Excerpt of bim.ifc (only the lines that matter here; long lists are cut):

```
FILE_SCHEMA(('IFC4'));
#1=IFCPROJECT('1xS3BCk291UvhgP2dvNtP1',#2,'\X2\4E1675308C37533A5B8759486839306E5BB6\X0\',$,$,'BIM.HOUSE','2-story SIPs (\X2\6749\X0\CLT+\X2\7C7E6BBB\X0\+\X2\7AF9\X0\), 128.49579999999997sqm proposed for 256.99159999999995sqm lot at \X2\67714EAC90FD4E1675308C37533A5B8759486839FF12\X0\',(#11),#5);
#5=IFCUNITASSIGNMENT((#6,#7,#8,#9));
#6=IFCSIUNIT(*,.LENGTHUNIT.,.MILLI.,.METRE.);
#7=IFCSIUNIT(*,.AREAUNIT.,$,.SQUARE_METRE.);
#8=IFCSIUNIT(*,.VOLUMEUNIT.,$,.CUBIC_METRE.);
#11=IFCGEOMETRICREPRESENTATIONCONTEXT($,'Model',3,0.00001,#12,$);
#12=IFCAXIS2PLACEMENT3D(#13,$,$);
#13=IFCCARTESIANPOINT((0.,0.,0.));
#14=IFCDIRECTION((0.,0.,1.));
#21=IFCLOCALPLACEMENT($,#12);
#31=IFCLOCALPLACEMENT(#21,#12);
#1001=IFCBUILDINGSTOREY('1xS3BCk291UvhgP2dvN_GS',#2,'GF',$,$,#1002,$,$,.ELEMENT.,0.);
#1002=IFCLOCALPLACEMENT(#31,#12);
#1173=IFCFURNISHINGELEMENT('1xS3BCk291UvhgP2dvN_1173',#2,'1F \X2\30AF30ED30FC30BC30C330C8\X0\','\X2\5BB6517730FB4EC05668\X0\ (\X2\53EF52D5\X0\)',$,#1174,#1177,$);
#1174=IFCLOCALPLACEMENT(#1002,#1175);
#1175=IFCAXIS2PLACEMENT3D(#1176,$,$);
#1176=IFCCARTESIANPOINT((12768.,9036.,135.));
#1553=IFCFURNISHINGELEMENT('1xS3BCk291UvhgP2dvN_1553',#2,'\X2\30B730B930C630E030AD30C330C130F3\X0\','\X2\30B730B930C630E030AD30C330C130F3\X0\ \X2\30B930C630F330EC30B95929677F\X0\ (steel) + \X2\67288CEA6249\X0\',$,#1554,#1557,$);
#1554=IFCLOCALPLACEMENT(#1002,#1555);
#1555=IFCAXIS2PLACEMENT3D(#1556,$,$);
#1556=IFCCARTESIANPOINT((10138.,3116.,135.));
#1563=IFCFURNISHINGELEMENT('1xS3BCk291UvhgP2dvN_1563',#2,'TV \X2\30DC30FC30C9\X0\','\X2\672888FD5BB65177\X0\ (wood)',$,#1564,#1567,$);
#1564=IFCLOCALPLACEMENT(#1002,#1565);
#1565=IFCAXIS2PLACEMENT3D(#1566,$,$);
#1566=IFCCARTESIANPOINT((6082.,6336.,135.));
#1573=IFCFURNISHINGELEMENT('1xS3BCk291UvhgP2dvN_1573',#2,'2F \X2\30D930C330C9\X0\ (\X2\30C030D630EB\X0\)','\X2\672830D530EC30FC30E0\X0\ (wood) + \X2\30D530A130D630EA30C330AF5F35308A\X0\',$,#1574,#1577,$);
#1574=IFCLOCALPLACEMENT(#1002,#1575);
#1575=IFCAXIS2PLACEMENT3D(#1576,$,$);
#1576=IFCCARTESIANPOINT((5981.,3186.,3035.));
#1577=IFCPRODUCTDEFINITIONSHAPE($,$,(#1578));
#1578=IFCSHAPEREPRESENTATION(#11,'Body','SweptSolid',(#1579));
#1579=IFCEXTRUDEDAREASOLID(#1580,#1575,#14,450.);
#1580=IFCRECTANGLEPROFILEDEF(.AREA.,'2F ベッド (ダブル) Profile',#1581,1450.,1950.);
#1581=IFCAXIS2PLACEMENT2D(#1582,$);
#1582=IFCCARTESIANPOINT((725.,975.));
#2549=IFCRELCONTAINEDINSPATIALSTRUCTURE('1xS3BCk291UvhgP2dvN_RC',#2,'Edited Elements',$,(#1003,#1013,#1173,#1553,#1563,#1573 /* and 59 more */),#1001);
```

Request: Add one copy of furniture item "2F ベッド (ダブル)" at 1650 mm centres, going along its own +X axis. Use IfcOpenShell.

```python
import ifcopenshell
import ifcopenshell.api.geometry
import ifcopenshell.api.root
import ifcopenshell.util.element
import ifcopenshell.util.placement

model = ifcopenshell.open("bim.ifc")


def reuse_history(source, copy):
    """copy_class also copies each property set's owner history, people and application; keep the originals."""
    for rel in copy.IsDefinedBy:
        if rel.is_a("IfcRelDefinesByProperties") and (history := rel.RelatingPropertyDefinition.OwnerHistory):
            rel.RelatingPropertyDefinition.OwnerHistory = source.OwnerHistory
            ifcopenshell.util.element.remove_deep2(model, history)


source = model.by_id(1573)
base = ifcopenshell.util.placement.get_local_placement(source.ObjectPlacement)
step = base[:3, 0] * 1650.0

for i in range(1, 2):
    copy = ifcopenshell.api.root.copy_class(model, product=source)
    copy.Representation = ifcopenshell.util.element.copy_deep(
        model, source.Representation, exclude=["IfcGeometricRepresentationContext", "IfcRepresentationMap"]
    )
    reuse_history(source, copy)
    matrix = base.copy()
    matrix[:3, 3] += i * step
    print("added at", matrix[:3, 3].round(3) + 0.0)
    ifcopenshell.api.geometry.edit_object_placement(model, product=copy, matrix=matrix, is_si=False)

model.write("bim_updated.ifc")
```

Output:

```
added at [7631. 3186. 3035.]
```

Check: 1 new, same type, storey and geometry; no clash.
